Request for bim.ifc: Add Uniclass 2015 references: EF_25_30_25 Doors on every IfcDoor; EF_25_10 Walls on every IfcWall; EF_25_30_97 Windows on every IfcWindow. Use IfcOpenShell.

First a look at what the model holds.

```python
import ifcopenshell

model = ifcopenshell.open("bim.ifc")
print(model.schema)
print("classifications:", [c.Name for c in model.by_type("IfcClassification")])
for ifc_class in ("IfcDoor", "IfcRoof", "IfcStair", "IfcWall", "IfcWindow"):
    print(ifc_class, len(model.by_type(ifc_class)))
```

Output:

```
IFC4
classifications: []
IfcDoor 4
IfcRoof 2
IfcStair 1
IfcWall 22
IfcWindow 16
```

```python
import ifcopenshell
import ifcopenshell.api.classification

model = ifcopenshell.open("bim.ifc")

system = ifcopenshell.api.classification.add_classification(model, classification="Uniclass 2015")

codes = {
    "IfcDoor": ("EF_25_30_25", "Doors"),
    "IfcWall": ("EF_25_10", "Walls"),
    "IfcWindow": ("EF_25_30_97", "Windows"),
}
for ifc_class, (code, name) in codes.items():
    products = model.by_type(ifc_class)
    ifcopenshell.api.classification.add_reference(
        model, products=products, classification=system, identification=code, name=name
    )
    print(code, len(products))

model.write("bim_updated.ifc")
```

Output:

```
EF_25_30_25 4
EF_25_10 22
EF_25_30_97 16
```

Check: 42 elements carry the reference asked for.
